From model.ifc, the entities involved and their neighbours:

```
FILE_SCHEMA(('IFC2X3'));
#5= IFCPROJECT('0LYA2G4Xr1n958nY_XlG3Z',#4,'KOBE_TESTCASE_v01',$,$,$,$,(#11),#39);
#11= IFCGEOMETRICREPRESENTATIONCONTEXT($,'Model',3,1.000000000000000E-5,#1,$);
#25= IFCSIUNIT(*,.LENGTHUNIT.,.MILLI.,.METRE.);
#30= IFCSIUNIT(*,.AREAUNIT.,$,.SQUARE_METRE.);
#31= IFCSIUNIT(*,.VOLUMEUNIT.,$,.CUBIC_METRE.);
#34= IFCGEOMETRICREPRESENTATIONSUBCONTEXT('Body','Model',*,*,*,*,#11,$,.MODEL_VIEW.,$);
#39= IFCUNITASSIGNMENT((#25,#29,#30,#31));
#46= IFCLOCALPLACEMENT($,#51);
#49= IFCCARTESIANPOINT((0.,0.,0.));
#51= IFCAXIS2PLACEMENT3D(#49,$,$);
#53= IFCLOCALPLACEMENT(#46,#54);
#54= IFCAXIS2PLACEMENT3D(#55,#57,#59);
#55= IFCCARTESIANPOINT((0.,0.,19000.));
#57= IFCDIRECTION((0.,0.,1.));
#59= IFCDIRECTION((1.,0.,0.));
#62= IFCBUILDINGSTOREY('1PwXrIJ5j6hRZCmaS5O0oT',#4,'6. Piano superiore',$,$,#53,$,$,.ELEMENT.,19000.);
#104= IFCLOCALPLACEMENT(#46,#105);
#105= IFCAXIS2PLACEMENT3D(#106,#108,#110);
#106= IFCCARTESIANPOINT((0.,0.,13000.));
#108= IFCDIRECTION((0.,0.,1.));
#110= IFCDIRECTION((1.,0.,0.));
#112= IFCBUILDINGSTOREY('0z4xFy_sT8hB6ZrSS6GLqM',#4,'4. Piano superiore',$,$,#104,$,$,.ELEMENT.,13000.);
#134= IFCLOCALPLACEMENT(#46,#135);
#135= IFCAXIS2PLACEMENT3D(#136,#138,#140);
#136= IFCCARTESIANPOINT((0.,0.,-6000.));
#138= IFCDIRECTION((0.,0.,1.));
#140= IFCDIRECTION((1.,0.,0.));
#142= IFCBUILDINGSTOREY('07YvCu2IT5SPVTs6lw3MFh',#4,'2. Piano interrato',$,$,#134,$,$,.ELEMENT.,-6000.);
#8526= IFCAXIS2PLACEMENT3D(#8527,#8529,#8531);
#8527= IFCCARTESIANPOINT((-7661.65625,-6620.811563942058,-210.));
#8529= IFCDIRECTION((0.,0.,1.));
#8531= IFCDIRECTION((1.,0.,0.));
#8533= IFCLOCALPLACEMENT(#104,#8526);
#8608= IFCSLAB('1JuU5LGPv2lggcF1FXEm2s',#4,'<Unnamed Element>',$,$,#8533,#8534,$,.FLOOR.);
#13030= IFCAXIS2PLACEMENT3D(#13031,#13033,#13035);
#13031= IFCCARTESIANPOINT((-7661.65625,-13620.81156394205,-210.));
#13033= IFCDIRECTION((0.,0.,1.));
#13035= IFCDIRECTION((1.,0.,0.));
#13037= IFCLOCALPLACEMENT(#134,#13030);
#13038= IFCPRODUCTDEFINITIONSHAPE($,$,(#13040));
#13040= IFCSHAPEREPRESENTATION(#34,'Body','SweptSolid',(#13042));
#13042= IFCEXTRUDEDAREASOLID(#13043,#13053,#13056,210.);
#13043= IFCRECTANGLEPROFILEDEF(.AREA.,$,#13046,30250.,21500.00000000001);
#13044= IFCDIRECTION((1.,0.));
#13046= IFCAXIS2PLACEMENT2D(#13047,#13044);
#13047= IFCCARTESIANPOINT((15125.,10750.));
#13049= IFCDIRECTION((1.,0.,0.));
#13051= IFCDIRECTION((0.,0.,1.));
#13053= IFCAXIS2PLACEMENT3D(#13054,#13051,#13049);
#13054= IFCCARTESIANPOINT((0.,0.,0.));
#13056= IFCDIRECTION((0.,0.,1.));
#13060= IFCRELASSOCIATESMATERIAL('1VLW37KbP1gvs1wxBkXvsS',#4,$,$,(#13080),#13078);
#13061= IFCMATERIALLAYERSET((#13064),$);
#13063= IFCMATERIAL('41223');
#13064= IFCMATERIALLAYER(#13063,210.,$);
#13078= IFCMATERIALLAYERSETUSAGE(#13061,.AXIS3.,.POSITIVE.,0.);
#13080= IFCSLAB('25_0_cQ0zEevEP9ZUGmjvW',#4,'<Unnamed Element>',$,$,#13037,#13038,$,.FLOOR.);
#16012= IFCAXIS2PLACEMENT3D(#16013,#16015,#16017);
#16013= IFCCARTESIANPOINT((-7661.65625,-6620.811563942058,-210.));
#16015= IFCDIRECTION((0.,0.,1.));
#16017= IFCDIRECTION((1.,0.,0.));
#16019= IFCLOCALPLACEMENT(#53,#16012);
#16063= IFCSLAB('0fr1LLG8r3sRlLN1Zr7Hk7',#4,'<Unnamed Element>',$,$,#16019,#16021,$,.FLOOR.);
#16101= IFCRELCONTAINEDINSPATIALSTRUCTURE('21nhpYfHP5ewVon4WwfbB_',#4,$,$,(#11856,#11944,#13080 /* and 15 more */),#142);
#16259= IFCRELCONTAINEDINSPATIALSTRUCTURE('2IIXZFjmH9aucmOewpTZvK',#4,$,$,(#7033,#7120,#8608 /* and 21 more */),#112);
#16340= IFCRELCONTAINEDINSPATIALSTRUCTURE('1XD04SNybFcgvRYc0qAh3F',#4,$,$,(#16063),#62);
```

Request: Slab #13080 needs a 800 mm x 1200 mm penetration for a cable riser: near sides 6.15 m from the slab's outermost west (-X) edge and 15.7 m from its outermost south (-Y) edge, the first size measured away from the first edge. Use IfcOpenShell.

```python
import numpy as np
import ifcopenshell
import ifcopenshell.api.feature
import ifcopenshell.api.geometry
import ifcopenshell.api.root
import ifcopenshell.geom
import ifcopenshell.util.placement
import ifcopenshell.util.representation
import ifcopenshell.util.shape
import ifcopenshell.util.unit

model = ifcopenshell.open("model.ifc")
unit_scale = ifcopenshell.util.unit.calculate_unit_scale(model)
settings = ifcopenshell.geom.settings()


def volume(element):
    """Net volume in cubic metres, openings subtracted."""
    shape = ifcopenshell.geom.create_shape(settings, element)
    return ifcopenshell.util.shape.get_volume(shape.geometry)


slab = model.by_guid("25_0_cQ0zEevEP9ZUGmjvW")
before = volume(slab)

# Extent in the slab's own axes, in metres. The edges named are its -X and -Y sides.
slab_shape = ifcopenshell.geom.create_shape(settings, slab)
vertices = ifcopenshell.util.shape.get_vertices(slab_shape.geometry)
x_min, y_min, bottom = vertices.min(axis=0)
top = vertices[:, 2].max()

opening = ifcopenshell.api.root.create_entity(model, ifc_class="IfcOpeningElement", name="Cable riser opening")
context = ifcopenshell.util.representation.get_context(model, "Model", "Body", "MODEL_VIEW")
width, depth = 0.8, 1.2
outline = [(0.0, 0.0), (width, 0.0), (width, depth), (0.0, depth), (0.0, 0.0)]
# Overshoot both faces by 50 mm so the cut is clean.
shape = ifcopenshell.api.geometry.add_slab_representation(
    model, context=context, depth=top - bottom + 0.1, polyline=outline
)
ifcopenshell.api.geometry.assign_representation(model, product=opening, representation=shape)

matrix = ifcopenshell.util.placement.get_local_placement(slab.ObjectPlacement)
matrix[:, 3] = matrix @ np.append(np.array([x_min + 6.15, y_min + 15.7, bottom - 0.05]) / unit_scale, 1.0)
ifcopenshell.api.geometry.edit_object_placement(model, product=opening, matrix=matrix, is_si=False)
ifcopenshell.api.feature.add_feature(model, feature=opening, element=slab)

after = volume(slab)

print(f"slab volume {before:.3f} -> {after:.3f} m3")

model.write("model_edited.ifc")
```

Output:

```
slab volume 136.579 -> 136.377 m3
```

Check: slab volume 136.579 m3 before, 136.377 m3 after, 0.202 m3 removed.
